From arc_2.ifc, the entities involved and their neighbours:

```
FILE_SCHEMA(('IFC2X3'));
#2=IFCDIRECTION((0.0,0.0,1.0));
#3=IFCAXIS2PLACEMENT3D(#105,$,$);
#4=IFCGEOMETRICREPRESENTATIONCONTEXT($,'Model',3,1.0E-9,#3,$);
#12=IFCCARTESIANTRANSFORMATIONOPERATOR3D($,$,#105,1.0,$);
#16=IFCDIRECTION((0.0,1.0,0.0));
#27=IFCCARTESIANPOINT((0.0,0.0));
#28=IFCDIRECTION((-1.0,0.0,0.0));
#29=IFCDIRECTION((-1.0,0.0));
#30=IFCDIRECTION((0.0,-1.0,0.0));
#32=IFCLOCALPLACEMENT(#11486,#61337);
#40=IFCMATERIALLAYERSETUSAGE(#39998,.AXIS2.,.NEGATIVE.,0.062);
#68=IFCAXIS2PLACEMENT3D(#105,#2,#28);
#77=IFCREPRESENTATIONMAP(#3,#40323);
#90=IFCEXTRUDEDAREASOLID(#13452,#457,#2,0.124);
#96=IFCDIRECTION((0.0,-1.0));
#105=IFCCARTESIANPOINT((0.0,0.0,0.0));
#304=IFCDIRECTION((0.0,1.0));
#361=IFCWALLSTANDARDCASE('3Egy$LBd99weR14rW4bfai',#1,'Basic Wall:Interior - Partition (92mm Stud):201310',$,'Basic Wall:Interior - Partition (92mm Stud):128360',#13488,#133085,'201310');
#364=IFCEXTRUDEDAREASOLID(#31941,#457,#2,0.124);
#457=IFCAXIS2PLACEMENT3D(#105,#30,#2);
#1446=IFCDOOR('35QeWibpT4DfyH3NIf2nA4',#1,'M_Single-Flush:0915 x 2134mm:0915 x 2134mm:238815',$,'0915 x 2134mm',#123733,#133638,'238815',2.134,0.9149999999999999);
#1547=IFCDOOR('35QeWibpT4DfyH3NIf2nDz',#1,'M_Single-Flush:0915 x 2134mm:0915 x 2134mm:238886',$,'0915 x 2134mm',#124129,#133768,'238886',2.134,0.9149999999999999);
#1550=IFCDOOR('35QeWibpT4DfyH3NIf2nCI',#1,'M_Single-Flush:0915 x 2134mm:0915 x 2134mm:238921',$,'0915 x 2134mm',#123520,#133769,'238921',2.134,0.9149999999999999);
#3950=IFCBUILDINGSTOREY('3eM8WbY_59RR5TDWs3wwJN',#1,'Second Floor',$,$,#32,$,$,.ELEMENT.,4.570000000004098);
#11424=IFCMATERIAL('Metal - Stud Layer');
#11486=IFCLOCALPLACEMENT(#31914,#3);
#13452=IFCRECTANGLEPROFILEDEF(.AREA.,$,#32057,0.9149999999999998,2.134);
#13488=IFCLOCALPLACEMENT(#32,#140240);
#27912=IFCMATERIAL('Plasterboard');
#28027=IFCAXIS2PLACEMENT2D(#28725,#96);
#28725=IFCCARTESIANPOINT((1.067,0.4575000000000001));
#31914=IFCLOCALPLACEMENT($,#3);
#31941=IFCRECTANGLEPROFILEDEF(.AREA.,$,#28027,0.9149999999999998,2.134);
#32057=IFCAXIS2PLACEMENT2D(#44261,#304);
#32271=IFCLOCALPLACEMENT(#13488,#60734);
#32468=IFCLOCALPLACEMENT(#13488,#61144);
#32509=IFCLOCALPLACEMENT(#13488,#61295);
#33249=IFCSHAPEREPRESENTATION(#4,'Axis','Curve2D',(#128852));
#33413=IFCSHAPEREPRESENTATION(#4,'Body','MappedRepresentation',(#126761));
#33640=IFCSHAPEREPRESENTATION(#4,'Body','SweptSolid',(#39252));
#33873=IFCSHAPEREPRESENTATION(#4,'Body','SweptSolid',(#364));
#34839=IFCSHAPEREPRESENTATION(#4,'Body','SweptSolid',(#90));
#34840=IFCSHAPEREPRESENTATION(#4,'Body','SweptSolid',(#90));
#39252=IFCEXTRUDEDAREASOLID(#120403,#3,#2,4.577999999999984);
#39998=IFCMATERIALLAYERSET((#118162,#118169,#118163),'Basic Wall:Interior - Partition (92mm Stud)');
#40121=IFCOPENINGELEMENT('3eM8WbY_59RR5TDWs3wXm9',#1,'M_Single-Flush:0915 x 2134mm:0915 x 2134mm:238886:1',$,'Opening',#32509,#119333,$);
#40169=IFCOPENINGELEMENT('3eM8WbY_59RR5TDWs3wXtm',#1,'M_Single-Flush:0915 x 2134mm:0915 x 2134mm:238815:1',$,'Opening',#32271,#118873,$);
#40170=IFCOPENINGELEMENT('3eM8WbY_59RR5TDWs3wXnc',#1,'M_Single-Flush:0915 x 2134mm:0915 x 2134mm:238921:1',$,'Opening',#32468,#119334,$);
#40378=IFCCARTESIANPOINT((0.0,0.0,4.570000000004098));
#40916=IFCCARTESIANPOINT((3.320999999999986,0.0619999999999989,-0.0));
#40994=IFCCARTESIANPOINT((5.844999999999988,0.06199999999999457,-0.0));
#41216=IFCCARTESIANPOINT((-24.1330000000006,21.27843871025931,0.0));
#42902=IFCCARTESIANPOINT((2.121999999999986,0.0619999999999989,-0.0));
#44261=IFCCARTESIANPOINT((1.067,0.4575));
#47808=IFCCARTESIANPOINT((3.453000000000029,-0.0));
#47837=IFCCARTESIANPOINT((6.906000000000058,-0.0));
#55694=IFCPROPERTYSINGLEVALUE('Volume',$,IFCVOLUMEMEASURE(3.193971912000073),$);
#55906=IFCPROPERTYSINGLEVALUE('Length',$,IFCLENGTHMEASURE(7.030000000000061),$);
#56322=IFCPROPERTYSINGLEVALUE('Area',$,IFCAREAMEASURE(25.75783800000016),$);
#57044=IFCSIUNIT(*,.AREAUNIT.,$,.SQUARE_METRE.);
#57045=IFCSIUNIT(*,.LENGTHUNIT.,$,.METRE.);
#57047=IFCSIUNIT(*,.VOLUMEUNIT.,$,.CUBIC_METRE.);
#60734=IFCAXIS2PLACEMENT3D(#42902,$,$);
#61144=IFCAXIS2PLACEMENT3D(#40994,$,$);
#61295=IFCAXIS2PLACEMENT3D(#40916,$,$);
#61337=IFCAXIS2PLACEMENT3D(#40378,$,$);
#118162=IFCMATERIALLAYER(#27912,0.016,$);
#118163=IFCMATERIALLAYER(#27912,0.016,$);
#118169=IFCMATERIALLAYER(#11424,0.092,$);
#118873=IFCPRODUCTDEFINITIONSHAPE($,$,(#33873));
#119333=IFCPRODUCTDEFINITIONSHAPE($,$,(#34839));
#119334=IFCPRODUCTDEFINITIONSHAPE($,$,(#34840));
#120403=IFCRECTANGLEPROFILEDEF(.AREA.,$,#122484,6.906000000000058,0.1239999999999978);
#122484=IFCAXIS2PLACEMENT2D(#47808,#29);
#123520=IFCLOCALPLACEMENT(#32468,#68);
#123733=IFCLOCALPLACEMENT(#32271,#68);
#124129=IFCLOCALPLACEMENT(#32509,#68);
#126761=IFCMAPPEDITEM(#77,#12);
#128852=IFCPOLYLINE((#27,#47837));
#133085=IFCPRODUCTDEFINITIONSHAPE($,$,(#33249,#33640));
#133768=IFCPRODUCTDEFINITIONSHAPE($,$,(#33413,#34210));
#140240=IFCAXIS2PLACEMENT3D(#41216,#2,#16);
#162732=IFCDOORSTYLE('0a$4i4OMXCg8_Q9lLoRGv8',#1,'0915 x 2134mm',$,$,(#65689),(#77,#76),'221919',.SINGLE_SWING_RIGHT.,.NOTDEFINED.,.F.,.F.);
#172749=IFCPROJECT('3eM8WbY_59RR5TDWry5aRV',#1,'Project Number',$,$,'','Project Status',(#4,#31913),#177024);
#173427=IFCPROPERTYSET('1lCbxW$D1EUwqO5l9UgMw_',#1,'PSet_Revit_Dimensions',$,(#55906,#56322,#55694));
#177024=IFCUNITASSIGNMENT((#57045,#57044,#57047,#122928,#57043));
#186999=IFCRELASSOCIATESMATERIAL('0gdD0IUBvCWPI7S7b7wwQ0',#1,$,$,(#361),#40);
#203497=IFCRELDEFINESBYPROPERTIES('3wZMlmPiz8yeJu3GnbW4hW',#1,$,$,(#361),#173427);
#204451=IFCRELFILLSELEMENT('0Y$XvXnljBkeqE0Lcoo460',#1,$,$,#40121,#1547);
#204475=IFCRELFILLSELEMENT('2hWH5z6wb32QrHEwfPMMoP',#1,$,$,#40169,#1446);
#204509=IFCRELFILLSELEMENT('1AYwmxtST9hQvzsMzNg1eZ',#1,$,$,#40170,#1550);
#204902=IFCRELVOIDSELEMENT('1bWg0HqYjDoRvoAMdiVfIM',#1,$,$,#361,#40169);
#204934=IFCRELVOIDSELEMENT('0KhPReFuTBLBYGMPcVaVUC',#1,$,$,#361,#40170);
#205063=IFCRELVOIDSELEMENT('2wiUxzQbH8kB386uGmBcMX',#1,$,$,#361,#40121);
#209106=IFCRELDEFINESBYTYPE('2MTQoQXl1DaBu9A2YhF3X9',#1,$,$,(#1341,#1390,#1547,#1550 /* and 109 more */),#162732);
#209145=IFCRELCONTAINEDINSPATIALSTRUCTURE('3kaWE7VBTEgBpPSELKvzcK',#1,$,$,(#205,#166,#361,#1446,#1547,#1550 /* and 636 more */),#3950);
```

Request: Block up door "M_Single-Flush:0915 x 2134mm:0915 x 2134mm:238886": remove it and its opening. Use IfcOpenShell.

```python
import ifcopenshell
import ifcopenshell.api.feature
import ifcopenshell.api.pset
import ifcopenshell.api.root
import ifcopenshell.geom
import ifcopenshell.util.element
import ifcopenshell.util.shape
import ifcopenshell.util.unit

model = ifcopenshell.open("arc_2.ifc")
area_scale = ifcopenshell.util.unit.calculate_unit_scale(model, "AREAUNIT")
volume_scale = ifcopenshell.util.unit.calculate_unit_scale(model, "VOLUMEUNIT")
settings = ifcopenshell.geom.settings()


def volume(element):
    """Net volume in cubic metres, openings subtracted."""
    shape = ifcopenshell.geom.create_shape(settings, element)
    return ifcopenshell.util.shape.get_volume(shape.geometry)


door = model.by_guid("35QeWibpT4DfyH3NIf2nDz")
opening = door.FillsVoids[0].RelatingOpeningElement
wall = opening.VoidsElements[0].RelatingBuildingElement
before = volume(wall)

ifcopenshell.api.root.remove_product(model, product=door)
ifcopenshell.api.feature.remove_feature(model, feature=opening)

after = volume(wall)
thickness = 0.124  # wall thickness in metres

# Update the wall's stored quantities.
pset = model.by_id(ifcopenshell.util.element.get_pset(wall, "PSet_Revit_Dimensions", should_inherit=False)["id"])
ifcopenshell.api.pset.edit_pset(model, pset=pset, properties={
    "Area": model.create_entity("IfcAreaMeasure", after / thickness / area_scale),
    "Volume": model.create_entity("IfcVolumeMeasure", after / volume_scale),
})

print(f"wall volume {before:.3f} -> {after:.3f} m3")

model.write("arc_2_edited.ifc")
```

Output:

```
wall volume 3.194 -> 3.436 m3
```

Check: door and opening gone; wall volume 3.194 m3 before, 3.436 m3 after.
